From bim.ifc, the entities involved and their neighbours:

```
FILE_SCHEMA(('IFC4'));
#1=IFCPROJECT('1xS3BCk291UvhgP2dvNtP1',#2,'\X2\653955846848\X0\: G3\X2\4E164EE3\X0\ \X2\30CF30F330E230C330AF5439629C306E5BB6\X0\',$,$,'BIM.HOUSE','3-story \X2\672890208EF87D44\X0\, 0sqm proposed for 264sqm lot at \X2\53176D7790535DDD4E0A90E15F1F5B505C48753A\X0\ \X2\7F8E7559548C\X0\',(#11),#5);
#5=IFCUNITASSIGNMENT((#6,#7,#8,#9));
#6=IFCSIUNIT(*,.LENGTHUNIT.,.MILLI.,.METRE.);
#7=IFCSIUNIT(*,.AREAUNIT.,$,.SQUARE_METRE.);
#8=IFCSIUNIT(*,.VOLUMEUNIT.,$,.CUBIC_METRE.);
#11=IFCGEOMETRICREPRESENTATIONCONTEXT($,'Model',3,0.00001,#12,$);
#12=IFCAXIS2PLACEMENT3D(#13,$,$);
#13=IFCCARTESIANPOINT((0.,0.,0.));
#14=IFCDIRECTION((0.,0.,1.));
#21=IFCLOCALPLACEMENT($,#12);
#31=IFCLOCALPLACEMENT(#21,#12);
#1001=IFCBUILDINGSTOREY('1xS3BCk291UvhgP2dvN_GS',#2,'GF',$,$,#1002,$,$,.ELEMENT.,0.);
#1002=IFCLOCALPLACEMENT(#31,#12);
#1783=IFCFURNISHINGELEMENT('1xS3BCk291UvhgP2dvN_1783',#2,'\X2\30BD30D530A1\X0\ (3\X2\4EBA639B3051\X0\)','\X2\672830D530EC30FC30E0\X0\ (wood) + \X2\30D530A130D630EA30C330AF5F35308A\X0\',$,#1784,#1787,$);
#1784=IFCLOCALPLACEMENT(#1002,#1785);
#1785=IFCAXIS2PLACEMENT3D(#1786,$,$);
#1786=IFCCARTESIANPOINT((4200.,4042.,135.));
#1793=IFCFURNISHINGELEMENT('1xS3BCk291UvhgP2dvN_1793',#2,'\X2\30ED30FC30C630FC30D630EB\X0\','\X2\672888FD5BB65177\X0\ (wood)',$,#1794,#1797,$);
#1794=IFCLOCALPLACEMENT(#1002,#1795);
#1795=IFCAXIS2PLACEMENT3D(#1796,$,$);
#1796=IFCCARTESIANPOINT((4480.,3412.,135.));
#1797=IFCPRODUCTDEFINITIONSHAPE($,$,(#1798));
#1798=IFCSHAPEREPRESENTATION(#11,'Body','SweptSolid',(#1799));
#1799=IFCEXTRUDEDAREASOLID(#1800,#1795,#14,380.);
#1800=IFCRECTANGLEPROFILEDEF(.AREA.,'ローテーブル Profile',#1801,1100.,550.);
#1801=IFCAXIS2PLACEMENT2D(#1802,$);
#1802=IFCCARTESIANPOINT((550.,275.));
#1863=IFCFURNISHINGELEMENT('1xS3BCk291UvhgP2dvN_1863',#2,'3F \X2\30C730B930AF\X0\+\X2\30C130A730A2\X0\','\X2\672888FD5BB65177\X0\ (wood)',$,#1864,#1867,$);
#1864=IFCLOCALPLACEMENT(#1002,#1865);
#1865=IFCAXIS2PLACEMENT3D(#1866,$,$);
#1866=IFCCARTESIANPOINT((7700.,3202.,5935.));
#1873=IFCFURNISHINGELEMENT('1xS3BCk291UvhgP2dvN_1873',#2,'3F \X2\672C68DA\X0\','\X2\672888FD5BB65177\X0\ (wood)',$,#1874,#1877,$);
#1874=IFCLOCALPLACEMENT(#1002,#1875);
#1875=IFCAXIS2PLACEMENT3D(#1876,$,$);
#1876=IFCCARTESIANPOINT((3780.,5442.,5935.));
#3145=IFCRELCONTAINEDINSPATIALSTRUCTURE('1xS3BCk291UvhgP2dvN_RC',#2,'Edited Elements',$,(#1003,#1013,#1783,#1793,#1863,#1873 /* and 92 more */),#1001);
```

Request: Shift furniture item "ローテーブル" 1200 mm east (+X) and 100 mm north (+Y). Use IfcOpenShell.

```python
import ifcopenshell
import ifcopenshell.api.geometry
import ifcopenshell.util.placement
import ifcopenshell.util.unit

model = ifcopenshell.open("bim.ifc")
unit_scale = ifcopenshell.util.unit.calculate_unit_scale(model)

item = model.by_guid("1xS3BCk291UvhgP2dvN_1793")
matrix = ifcopenshell.util.placement.get_local_placement(item.ObjectPlacement)
matrix[0, 3] += 1.2 / unit_scale
matrix[1, 3] += 0.1 / unit_scale
ifcopenshell.api.geometry.edit_object_placement(model, product=item, matrix=matrix, is_si=False)

print(ifcopenshell.util.placement.get_local_placement(item.ObjectPlacement).round(3) + 0.0)

model.write("bim_rev.ifc")
```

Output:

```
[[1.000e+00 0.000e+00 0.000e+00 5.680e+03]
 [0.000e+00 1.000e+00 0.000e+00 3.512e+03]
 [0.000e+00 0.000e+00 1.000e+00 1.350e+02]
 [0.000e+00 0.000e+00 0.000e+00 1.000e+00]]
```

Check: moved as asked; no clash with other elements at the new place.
